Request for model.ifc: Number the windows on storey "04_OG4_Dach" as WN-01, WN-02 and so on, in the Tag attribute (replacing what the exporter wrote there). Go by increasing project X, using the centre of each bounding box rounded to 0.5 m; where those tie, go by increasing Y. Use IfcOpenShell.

First a look at what the model holds.

```python
import ifcopenshell
import ifcopenshell.util.element
import ifcopenshell.util.placement

model = ifcopenshell.open("model.ifc")
print(model.schema)
storey = next(s for s in model.by_type("IfcBuildingStorey") if s.Name == "04_OG4_Dach")
windows = [e for e in ifcopenshell.util.element.get_decomposition(storey) if e.is_a("IfcWindow")]
for e in sorted(windows, key=lambda e: e.id()):
    origin = ifcopenshell.util.placement.get_local_placement(e.ObjectPlacement)[:3, 3]
    print(e.id(), e.Tag, e.Name, origin.round(2) + 0.0, sep=" | ")
```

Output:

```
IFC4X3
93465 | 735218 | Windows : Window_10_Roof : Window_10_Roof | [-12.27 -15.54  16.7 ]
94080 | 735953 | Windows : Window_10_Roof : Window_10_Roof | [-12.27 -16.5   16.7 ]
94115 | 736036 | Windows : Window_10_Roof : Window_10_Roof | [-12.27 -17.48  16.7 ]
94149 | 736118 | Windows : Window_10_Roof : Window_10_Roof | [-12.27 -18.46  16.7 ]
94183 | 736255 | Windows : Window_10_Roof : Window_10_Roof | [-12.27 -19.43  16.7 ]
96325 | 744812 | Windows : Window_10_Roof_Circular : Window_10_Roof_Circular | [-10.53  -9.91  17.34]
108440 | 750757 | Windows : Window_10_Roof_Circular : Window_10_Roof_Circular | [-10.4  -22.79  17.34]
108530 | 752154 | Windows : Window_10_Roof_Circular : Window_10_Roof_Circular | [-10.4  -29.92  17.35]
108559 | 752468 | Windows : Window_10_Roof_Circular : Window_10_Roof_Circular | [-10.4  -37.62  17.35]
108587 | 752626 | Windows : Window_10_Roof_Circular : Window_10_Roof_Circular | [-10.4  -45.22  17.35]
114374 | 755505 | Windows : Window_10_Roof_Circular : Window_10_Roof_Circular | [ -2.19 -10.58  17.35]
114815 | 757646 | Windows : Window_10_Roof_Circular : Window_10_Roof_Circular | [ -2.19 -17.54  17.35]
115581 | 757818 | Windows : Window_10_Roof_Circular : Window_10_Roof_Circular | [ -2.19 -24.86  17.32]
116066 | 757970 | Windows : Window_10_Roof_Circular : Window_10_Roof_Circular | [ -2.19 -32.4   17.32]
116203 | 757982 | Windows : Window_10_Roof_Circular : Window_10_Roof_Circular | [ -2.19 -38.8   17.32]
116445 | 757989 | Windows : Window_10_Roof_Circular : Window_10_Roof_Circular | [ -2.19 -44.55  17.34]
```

```python
import ifcopenshell
import ifcopenshell.geom
import ifcopenshell.util.element
import ifcopenshell.util.shape

model = ifcopenshell.open("model.ifc")
settings = ifcopenshell.geom.settings()
settings.set("use-world-coords", True)


def centre(element):
    shape = ifcopenshell.geom.create_shape(settings, element)
    return ifcopenshell.util.shape.get_bbox_centroid(shape.geometry)


storey = next(s for s in model.by_type("IfcBuildingStorey") if s.Name == "04_OG4_Dach")
windows = [e for e in ifcopenshell.util.element.get_decomposition(storey) if e.is_a("IfcWindow")]

# Insertion points can sit at a corner or the storey origin, so sort by the geometry (in metres).
centres = {e: centre(e) for e in windows}
windows.sort(key=lambda e: (round(centres[e][0] / 0.5), centres[e][1]))

for i, e in enumerate(windows, start=1):
    number = f"WN-{i:02d}"
    e.Tag = number
    print(e.id(), number)

model.write("model_updated.ifc")
```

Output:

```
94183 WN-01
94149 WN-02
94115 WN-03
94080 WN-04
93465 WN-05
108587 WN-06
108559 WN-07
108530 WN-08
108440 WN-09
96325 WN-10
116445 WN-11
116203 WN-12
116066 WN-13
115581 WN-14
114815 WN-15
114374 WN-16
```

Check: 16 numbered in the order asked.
